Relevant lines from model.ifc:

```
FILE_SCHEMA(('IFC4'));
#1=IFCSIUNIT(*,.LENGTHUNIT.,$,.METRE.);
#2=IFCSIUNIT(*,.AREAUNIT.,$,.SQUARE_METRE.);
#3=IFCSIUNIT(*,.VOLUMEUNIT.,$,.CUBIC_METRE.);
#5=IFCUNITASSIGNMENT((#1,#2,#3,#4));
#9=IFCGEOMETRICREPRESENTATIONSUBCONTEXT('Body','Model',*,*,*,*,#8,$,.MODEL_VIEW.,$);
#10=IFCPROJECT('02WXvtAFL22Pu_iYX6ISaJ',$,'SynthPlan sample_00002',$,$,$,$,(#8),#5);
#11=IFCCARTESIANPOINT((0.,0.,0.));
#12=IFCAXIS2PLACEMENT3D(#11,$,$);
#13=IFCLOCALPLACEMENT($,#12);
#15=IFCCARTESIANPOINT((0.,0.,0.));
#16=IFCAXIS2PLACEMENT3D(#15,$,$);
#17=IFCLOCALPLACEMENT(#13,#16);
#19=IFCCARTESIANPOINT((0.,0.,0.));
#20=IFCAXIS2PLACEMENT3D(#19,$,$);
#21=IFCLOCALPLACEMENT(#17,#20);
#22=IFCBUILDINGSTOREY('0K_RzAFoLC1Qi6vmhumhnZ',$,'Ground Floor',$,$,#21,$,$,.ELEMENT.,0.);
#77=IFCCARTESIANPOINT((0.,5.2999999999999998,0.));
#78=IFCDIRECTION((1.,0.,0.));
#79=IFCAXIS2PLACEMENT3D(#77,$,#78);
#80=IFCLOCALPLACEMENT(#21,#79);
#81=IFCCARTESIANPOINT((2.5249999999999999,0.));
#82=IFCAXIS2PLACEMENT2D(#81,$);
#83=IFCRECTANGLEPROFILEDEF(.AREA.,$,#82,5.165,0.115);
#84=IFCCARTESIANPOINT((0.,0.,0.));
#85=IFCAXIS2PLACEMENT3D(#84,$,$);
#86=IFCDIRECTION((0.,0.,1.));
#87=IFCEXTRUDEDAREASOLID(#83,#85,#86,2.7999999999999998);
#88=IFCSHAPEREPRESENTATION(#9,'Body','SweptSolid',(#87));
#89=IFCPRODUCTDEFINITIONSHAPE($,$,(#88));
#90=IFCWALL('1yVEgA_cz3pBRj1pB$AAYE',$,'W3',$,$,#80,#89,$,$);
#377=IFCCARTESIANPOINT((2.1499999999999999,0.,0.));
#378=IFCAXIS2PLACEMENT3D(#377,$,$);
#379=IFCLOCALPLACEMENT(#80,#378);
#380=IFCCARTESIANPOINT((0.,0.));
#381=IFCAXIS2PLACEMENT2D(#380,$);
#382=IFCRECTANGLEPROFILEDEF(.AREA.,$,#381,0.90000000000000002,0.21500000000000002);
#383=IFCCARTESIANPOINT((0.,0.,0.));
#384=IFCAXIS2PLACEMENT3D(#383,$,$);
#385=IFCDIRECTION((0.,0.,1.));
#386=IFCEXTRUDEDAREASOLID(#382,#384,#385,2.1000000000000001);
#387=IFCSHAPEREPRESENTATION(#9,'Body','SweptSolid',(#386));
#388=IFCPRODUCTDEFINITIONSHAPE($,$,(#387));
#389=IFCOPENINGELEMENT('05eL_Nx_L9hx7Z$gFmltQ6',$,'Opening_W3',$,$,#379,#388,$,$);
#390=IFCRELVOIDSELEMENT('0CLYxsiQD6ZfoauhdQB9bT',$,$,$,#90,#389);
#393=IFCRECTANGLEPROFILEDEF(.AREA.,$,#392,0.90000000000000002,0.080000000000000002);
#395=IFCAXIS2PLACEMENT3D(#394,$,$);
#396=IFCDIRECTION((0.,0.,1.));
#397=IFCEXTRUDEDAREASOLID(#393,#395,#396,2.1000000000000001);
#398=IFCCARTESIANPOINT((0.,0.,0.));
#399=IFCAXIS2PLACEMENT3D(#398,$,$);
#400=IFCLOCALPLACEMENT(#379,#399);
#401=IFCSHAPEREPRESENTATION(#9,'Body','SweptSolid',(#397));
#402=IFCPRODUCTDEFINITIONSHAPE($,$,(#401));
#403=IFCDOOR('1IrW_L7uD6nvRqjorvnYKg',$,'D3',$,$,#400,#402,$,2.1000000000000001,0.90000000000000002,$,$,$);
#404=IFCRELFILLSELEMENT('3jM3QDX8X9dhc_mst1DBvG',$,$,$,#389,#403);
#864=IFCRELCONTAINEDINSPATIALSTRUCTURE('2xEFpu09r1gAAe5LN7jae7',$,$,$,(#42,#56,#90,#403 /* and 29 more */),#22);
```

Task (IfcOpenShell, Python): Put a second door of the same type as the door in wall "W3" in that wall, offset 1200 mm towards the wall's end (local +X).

```python
import ifcopenshell
import ifcopenshell.api.feature
import ifcopenshell.api.geometry
import ifcopenshell.api.root
import ifcopenshell.geom
import ifcopenshell.util.element
import ifcopenshell.util.placement
import ifcopenshell.util.shape

model = ifcopenshell.open("model.ifc")
settings = ifcopenshell.geom.settings()


def volume(element):
    """Net volume in cubic metres, openings subtracted."""
    shape = ifcopenshell.geom.create_shape(settings, element)
    return ifcopenshell.util.shape.get_volume(shape.geometry)


door = model.by_guid("1IrW_L7uD6nvRqjorvnYKg")
opening = door.FillsVoids[0].RelatingOpeningElement
wall = opening.VoidsElements[0].RelatingBuildingElement
before = volume(wall)
shift = ifcopenshell.util.placement.get_local_placement(wall.ObjectPlacement)[:3, 0] * 1.2

# copy_class copies the void relationship, type, container and properties, but no geometry.
new_opening = ifcopenshell.api.root.copy_class(model, product=opening)
new_opening.Representation = ifcopenshell.util.element.copy_deep(
    model, opening.Representation, exclude=["IfcGeometricRepresentationContext", "IfcRepresentationMap"]
)
new_door = ifcopenshell.api.root.copy_class(model, product=door)
new_door.Representation = ifcopenshell.util.element.copy_deep(
    model, door.Representation, exclude=["IfcGeometricRepresentationContext", "IfcRepresentationMap"]
)
ifcopenshell.api.feature.add_filling(model, opening=new_opening, element=new_door)

for old, new in ((opening, new_opening), (door, new_door)):
    matrix = ifcopenshell.util.placement.get_local_placement(old.ObjectPlacement)
    matrix[:3, 3] += shift
    ifcopenshell.api.geometry.edit_object_placement(model, product=new, matrix=matrix, is_si=False)

after = volume(wall)

print(f"wall volume {before:.3f} -> {after:.3f} m3")

model.write("model_v2.ifc")
```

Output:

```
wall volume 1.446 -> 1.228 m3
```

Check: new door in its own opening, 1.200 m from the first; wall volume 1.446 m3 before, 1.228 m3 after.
